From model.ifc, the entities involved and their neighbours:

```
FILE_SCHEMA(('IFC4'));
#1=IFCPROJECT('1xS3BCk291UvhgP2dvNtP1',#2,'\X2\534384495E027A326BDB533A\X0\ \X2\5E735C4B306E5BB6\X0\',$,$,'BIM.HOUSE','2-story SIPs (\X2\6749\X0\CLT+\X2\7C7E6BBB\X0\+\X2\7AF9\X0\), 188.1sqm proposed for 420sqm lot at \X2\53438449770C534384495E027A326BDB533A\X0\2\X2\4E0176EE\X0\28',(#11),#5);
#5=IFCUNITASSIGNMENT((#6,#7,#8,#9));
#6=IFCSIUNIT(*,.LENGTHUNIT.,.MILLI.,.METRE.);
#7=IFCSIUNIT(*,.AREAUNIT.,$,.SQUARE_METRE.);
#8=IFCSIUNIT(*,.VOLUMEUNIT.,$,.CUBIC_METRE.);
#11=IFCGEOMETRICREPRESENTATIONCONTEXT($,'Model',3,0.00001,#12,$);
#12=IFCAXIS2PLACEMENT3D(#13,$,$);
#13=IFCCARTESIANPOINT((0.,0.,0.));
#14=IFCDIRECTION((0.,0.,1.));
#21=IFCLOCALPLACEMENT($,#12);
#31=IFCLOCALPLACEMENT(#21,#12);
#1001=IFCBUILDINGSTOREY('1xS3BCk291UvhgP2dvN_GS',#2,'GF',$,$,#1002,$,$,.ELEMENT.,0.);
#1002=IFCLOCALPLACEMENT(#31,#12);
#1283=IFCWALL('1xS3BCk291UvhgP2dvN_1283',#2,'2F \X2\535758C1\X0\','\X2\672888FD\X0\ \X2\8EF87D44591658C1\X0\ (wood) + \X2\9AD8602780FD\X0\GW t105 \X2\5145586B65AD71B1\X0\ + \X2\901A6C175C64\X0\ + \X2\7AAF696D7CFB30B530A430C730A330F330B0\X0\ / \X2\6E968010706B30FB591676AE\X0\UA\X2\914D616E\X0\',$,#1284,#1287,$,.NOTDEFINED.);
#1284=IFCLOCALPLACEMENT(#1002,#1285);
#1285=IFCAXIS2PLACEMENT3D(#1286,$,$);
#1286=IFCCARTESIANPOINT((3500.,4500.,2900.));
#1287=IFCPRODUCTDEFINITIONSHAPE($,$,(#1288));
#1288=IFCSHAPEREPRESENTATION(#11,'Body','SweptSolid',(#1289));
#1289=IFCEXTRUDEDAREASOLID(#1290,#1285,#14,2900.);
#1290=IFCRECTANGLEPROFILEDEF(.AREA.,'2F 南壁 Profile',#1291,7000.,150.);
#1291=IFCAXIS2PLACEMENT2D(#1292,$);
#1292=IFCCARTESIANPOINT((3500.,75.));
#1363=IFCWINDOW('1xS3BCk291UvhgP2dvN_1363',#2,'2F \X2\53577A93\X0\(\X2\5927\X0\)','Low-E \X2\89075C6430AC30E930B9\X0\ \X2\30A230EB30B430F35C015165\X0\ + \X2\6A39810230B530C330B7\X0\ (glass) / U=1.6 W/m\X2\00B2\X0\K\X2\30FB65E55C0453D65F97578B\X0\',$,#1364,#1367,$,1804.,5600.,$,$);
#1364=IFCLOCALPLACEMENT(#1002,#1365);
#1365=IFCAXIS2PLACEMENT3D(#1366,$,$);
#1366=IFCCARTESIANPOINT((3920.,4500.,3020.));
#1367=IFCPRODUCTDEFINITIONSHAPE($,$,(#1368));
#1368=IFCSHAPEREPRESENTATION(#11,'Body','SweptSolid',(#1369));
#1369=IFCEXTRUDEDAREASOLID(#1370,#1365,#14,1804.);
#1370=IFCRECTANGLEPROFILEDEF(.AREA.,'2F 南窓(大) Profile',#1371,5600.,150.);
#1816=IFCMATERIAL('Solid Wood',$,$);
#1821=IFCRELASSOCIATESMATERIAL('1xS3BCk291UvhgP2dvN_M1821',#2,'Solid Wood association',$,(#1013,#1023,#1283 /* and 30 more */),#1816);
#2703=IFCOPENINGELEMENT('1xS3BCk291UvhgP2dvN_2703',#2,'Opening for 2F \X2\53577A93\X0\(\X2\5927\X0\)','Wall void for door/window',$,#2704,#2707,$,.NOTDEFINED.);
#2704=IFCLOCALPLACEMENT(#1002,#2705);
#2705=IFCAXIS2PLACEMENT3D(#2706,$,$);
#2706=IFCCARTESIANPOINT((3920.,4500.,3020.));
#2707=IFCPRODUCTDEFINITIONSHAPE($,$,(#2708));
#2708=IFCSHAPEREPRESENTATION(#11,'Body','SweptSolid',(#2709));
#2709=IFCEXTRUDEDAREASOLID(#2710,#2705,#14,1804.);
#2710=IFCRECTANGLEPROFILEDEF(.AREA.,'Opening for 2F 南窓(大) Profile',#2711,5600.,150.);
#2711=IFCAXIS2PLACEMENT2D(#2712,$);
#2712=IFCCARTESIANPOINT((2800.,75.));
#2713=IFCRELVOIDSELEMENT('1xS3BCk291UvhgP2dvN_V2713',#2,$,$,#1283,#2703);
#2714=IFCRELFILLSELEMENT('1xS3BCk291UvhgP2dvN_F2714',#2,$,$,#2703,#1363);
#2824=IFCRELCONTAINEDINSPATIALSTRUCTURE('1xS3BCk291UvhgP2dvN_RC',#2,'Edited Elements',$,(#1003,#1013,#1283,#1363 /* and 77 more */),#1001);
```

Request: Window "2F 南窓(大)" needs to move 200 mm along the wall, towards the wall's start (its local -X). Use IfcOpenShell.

```python
import ifcopenshell
import ifcopenshell.api.geometry
import ifcopenshell.util.placement
import ifcopenshell.util.unit

model = ifcopenshell.open("model.ifc")
unit_scale = ifcopenshell.util.unit.calculate_unit_scale(model)

window = model.by_id(1363)
opening = window.FillsVoids[0].RelatingOpeningElement
wall = opening.VoidsElements[0].RelatingBuildingElement

wall_matrix = ifcopenshell.util.placement.get_local_placement(wall.ObjectPlacement)
shift = wall_matrix[:3, 0] * -0.2 / unit_scale
before = ifcopenshell.util.placement.get_local_placement(window.ObjectPlacement)[:3, 3].copy()

# The window is not placed relative to its opening, so move both.
for product in (opening, window):
    matrix = ifcopenshell.util.placement.get_local_placement(product.ObjectPlacement)
    matrix[:3, 3] += shift
    ifcopenshell.api.geometry.edit_object_placement(model, product=product, matrix=matrix, is_si=False)

after = ifcopenshell.util.placement.get_local_placement(window.ObjectPlacement)[:3, 3]
print("window moved by", (after - before).round(3) + 0.0)

model.write("model_edited.ifc")
```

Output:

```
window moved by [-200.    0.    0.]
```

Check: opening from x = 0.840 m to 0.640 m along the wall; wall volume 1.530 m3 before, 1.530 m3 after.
